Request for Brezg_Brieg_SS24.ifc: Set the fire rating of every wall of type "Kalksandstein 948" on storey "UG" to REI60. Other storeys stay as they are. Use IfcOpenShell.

First a look at what the model holds.

```python
import ifcopenshell
import ifcopenshell.util.element

model = ifcopenshell.open("Brezg_Brieg_SS24.ifc")
print(model.schema)
storey = next(s for s in model.by_type("IfcBuildingStorey") if s.Name == "UG")
walls = [e for e in ifcopenshell.util.element.get_decomposition(storey) if e.is_a("IfcWall")]
seen = {}
for e in walls:
    element_type = ifcopenshell.util.element.get_type(e)
    key = (element_type.Name if element_type != e and element_type else None, ifcopenshell.util.element.get_pset(e, "Pset_WallCommon", "FireRating"))
    seen[key] = seen.get(key, 0) + 1
for (name, value), count in sorted(seen.items(), key=str):
    print(count, "x", name, "|", value)
```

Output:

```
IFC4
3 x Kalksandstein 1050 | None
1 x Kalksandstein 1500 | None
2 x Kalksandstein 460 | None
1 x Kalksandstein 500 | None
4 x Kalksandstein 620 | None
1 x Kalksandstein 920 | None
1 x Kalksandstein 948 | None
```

```python
import ifcopenshell
import ifcopenshell.api.pset
import ifcopenshell.util.element

model = ifcopenshell.open("Brezg_Brieg_SS24.ifc")

storey = next(s for s in model.by_type("IfcBuildingStorey") if s.Name == "UG")
walls = [e for e in ifcopenshell.util.element.get_decomposition(storey) if e.is_a("IfcWall")]

count = 0
for e in walls:
    element_type = ifcopenshell.util.element.get_type(e)
    if element_type in (None, e) or element_type.Name != "Kalksandstein 948":
        continue
    # add_pset returns the element's existing set when there is one.
    pset = ifcopenshell.api.pset.add_pset(model, product=e, name="Pset_WallCommon")
    ifcopenshell.api.pset.edit_pset(model, pset=pset, properties={"FireRating": "REI60"})
    count += 1

print(count, "walls updated")

model.write("Brezg_Brieg_SS24_rev.ifc")
```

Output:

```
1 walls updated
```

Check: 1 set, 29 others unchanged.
